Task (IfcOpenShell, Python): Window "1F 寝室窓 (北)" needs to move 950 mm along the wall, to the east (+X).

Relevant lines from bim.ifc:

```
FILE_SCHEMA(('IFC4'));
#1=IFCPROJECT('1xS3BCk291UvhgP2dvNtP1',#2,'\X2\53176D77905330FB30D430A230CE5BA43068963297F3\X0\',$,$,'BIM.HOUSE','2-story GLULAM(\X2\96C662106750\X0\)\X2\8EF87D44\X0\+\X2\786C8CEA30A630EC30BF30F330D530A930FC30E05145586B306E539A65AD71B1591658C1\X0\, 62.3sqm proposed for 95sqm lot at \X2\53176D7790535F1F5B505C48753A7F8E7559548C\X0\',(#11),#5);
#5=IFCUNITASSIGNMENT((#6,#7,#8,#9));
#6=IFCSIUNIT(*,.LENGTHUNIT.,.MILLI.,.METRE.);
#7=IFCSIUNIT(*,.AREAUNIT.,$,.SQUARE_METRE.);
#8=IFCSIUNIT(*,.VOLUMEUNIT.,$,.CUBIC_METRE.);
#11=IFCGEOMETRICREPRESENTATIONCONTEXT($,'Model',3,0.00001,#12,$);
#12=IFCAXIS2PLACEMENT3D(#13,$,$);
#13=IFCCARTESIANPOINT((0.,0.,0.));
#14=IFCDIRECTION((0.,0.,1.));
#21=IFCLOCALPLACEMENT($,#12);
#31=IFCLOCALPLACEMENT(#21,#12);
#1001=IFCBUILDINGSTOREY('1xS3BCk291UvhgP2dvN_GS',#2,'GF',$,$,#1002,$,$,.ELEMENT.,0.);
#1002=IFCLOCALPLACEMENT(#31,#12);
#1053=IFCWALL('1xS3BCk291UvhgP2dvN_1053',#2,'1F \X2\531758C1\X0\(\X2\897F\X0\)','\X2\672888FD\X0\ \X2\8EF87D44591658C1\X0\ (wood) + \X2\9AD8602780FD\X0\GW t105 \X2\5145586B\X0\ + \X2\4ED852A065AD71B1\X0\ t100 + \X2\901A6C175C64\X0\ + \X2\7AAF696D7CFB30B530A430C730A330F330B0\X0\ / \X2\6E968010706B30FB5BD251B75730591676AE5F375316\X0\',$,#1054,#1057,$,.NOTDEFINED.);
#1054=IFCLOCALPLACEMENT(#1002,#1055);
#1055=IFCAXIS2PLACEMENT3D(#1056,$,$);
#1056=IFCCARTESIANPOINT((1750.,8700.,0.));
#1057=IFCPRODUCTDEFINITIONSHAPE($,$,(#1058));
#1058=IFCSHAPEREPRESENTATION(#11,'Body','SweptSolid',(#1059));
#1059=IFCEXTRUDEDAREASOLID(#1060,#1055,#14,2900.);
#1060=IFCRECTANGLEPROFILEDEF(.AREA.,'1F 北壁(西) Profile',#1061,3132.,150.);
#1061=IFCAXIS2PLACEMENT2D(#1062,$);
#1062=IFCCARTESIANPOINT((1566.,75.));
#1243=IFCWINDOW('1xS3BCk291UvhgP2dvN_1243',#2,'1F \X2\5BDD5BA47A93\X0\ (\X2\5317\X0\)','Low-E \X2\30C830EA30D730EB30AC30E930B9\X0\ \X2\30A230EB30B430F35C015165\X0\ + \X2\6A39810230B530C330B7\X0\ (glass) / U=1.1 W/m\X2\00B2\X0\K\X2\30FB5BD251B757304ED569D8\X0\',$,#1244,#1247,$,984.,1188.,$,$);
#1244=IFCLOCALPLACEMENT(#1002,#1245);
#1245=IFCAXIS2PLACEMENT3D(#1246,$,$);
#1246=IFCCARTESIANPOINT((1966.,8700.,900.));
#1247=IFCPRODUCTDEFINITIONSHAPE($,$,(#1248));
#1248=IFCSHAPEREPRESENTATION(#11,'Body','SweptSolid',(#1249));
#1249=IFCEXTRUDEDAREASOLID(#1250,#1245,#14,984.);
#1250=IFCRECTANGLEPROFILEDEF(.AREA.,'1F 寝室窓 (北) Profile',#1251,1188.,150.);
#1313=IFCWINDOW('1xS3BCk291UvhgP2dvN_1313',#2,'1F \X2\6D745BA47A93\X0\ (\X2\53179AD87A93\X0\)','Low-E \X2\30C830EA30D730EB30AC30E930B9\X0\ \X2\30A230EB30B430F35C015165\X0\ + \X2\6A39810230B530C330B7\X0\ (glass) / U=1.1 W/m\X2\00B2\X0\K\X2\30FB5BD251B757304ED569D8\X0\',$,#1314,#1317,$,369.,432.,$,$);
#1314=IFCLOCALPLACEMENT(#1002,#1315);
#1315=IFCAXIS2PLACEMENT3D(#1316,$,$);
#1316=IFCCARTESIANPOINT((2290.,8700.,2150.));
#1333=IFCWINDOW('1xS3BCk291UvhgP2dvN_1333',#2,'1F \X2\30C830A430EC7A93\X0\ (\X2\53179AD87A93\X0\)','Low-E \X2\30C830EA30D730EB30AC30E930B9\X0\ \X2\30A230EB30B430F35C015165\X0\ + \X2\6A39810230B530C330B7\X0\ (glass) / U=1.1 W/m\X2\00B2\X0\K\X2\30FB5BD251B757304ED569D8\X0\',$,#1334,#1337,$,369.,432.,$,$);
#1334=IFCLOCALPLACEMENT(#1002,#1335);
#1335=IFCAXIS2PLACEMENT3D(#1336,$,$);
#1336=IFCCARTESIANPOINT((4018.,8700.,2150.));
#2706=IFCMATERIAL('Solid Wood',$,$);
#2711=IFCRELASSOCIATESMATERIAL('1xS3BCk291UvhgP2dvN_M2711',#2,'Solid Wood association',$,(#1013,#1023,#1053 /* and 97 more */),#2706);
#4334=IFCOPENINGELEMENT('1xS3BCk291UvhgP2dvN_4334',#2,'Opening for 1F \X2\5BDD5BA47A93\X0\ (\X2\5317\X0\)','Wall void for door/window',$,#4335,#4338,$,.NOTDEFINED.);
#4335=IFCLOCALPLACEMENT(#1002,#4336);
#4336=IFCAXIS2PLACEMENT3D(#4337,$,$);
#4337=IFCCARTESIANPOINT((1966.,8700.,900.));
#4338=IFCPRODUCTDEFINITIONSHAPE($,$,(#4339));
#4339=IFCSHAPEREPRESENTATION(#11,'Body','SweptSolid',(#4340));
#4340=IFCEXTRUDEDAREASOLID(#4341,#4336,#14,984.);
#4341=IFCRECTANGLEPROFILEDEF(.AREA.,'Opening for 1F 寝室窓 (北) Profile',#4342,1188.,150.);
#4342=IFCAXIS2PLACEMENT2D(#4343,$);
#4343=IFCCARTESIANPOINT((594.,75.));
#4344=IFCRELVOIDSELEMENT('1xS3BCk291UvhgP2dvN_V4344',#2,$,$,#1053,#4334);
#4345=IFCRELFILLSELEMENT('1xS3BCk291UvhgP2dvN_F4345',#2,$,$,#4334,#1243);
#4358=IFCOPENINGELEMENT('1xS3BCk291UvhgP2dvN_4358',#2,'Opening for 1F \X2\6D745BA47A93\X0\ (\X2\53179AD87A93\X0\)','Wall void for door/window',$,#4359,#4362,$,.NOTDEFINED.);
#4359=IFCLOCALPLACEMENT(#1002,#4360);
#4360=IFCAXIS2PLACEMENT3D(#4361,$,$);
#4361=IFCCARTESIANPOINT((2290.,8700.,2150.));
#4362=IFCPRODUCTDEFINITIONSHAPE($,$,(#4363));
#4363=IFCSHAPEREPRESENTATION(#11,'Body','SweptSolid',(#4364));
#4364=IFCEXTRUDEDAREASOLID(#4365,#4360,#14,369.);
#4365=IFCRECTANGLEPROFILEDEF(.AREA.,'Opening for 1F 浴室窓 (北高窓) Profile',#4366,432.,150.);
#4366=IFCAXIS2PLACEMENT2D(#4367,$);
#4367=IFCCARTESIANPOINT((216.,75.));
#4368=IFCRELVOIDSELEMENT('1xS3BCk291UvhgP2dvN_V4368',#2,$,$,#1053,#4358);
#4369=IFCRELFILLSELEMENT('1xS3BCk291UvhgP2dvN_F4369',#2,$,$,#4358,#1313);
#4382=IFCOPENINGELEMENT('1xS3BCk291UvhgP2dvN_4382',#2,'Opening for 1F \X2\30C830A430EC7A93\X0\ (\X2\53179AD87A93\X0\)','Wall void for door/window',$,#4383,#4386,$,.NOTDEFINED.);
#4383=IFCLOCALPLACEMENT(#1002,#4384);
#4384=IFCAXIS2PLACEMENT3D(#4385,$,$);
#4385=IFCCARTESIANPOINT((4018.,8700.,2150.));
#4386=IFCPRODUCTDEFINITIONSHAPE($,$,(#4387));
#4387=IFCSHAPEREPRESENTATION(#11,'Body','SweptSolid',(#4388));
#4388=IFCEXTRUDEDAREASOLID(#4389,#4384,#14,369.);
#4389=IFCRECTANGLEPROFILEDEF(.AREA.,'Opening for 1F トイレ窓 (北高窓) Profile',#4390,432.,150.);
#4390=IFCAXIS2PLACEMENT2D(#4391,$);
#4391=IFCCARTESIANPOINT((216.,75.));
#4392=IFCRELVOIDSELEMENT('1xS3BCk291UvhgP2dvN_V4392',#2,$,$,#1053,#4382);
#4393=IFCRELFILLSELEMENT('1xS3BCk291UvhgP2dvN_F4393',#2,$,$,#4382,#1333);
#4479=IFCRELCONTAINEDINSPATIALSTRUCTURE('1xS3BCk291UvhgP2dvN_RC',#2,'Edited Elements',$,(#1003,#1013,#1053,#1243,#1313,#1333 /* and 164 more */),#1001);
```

```python
import ifcopenshell
import ifcopenshell.api.geometry
import ifcopenshell.util.placement
import ifcopenshell.util.unit

model = ifcopenshell.open("bim.ifc")
unit_scale = ifcopenshell.util.unit.calculate_unit_scale(model)

window = model.by_guid("1xS3BCk291UvhgP2dvN_1243")
opening = window.FillsVoids[0].RelatingOpeningElement
wall = opening.VoidsElements[0].RelatingBuildingElement

wall_matrix = ifcopenshell.util.placement.get_local_placement(wall.ObjectPlacement)
shift = wall_matrix[:3, 0] * 0.95 / unit_scale
before = ifcopenshell.util.placement.get_local_placement(window.ObjectPlacement)[:3, 3].copy()

# The window is not placed relative to its opening, so move both.
for product in (opening, window):
    matrix = ifcopenshell.util.placement.get_local_placement(product.ObjectPlacement)
    matrix[:3, 3] += shift
    ifcopenshell.api.geometry.edit_object_placement(model, product=product, matrix=matrix, is_si=False)

after = ifcopenshell.util.placement.get_local_placement(window.ObjectPlacement)[:3, 3]
print("window moved by", (after - before).round(3) + 0.0)

model.write("bim_edited.ifc")
```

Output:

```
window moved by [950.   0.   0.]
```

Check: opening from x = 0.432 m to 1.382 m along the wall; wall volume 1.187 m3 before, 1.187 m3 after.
